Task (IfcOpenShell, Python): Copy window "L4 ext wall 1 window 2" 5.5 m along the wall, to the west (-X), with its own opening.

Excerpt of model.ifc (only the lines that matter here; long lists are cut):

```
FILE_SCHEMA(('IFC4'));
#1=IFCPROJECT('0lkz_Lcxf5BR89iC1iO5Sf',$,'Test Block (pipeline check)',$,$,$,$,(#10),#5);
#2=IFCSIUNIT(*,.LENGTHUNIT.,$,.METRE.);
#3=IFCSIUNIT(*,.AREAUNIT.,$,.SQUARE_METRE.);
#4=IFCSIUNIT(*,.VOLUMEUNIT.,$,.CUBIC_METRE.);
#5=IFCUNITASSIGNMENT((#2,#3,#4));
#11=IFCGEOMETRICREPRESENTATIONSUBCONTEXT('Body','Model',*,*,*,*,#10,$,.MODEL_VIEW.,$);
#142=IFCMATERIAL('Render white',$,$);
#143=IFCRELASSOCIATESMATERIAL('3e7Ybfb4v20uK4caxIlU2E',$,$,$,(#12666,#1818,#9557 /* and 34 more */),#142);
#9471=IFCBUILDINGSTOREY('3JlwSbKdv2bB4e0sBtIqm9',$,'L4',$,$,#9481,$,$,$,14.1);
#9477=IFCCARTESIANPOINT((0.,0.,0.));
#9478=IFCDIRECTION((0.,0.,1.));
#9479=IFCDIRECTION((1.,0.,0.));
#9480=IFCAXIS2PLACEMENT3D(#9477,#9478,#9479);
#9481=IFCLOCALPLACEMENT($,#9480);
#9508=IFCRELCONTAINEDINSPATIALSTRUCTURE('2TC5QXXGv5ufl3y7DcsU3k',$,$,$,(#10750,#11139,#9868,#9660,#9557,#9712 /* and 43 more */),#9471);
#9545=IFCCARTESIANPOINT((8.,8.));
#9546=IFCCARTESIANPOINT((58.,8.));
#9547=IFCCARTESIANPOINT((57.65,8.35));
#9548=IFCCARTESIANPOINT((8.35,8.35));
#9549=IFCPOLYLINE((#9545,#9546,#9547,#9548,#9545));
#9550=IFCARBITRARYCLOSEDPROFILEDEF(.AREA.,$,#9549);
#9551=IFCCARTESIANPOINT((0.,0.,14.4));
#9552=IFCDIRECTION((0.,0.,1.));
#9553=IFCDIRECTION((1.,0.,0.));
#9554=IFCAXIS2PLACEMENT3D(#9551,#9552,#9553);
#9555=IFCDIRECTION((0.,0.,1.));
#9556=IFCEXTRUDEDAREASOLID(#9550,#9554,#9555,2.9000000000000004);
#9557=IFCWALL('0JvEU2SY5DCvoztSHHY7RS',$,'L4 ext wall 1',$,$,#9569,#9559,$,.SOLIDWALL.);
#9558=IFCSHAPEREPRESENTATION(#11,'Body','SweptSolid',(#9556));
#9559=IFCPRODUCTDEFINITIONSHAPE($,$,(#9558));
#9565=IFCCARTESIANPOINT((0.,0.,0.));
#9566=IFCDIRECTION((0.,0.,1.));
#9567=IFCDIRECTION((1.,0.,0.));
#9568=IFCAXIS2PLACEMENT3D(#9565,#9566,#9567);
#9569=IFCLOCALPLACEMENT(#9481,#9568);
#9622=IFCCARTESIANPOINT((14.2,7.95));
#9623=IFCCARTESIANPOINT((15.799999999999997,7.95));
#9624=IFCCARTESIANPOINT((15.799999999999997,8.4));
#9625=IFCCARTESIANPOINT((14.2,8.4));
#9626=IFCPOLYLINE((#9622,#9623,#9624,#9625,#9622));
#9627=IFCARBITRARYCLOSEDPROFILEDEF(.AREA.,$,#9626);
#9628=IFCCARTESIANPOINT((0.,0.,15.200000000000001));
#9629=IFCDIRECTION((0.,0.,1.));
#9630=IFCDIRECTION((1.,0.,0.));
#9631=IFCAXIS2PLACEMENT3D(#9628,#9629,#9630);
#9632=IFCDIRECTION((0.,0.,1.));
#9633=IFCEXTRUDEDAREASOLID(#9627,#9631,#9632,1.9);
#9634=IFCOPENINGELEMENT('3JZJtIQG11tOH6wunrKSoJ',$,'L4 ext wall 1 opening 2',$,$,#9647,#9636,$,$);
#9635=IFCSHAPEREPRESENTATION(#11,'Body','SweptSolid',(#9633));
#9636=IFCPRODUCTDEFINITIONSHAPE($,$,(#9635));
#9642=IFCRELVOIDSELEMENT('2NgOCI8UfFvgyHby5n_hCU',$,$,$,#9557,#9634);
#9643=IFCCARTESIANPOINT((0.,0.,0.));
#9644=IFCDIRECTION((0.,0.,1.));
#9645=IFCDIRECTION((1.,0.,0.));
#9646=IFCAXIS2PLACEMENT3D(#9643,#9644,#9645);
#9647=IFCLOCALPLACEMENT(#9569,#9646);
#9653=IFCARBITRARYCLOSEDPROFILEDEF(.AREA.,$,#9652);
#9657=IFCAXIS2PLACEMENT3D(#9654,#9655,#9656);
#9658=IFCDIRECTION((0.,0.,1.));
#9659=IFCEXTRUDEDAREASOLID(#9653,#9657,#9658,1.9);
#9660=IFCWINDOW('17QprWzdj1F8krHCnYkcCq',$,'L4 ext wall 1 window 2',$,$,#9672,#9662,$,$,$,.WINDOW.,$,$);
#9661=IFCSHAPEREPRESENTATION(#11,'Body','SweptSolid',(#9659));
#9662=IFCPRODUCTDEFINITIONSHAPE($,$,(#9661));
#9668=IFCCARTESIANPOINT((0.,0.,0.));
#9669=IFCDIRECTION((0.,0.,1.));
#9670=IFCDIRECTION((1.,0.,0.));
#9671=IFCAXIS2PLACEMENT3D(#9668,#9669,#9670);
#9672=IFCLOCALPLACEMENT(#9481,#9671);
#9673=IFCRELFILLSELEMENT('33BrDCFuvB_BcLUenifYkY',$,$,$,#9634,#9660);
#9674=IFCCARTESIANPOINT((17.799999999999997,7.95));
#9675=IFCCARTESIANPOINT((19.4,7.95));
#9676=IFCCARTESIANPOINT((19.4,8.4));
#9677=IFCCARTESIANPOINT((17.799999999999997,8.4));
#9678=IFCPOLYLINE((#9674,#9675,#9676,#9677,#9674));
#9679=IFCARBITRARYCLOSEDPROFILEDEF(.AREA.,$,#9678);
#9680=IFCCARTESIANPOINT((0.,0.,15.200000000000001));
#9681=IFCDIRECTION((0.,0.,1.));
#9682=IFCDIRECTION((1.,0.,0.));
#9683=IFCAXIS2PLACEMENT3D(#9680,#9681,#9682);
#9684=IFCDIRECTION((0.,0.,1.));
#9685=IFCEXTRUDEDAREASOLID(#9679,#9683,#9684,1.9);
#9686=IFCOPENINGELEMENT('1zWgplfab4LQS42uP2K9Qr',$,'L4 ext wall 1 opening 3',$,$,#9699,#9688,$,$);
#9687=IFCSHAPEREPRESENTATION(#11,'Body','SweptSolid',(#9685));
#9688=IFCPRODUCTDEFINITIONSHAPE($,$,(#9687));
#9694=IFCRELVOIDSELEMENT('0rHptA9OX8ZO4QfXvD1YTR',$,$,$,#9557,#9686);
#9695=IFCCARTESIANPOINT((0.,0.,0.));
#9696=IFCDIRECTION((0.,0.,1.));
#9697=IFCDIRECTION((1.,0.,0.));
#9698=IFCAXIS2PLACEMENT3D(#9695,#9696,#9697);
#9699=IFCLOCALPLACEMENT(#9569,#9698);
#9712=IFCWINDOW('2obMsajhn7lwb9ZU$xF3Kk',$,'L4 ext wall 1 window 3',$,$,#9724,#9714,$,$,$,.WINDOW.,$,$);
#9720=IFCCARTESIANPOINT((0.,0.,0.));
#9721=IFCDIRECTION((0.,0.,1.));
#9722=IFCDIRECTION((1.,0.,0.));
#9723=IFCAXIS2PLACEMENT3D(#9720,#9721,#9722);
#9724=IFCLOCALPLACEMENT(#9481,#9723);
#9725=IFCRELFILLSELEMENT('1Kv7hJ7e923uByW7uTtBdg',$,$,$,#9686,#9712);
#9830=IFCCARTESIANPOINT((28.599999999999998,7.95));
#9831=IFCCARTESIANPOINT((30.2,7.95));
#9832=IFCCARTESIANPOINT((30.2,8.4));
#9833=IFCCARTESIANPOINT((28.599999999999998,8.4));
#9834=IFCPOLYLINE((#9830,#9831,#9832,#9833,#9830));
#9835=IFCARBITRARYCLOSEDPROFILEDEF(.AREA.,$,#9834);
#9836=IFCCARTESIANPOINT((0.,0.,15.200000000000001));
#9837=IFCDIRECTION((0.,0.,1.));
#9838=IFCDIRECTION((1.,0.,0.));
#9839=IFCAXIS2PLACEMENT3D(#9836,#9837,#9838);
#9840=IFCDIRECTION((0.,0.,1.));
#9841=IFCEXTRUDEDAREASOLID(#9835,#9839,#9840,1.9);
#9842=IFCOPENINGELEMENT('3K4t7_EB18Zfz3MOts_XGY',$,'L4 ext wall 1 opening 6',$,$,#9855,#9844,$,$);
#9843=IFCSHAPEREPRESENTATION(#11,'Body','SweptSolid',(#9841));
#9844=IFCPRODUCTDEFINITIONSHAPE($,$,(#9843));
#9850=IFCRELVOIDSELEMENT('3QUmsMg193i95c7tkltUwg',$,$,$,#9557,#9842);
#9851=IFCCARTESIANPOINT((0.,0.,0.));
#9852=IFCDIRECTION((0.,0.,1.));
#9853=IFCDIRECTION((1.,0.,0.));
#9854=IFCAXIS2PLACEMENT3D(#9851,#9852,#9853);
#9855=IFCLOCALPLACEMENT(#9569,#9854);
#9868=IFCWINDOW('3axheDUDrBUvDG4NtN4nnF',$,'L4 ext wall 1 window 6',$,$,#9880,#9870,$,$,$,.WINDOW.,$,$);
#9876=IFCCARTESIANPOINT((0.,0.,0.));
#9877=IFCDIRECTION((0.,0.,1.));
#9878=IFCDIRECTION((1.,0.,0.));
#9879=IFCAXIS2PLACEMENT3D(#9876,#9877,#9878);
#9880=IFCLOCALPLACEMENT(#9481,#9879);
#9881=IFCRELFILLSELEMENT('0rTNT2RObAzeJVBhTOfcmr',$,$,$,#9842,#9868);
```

```python
import ifcopenshell
import ifcopenshell.api.feature
import ifcopenshell.api.geometry
import ifcopenshell.api.root
import ifcopenshell.geom
import ifcopenshell.util.element
import ifcopenshell.util.placement
import ifcopenshell.util.shape
import ifcopenshell.util.unit

model = ifcopenshell.open("model.ifc")
unit_scale = ifcopenshell.util.unit.calculate_unit_scale(model)
settings = ifcopenshell.geom.settings()


def volume(element):
    """Net volume in cubic metres, openings subtracted."""
    shape = ifcopenshell.geom.create_shape(settings, element)
    return ifcopenshell.util.shape.get_volume(shape.geometry)


window = model.by_id(9660)
opening = window.FillsVoids[0].RelatingOpeningElement
wall = opening.VoidsElements[0].RelatingBuildingElement
before = volume(wall)
shift = ifcopenshell.util.placement.get_local_placement(wall.ObjectPlacement)[:3, 0] * -5.5 / unit_scale

# copy_class copies the void relationship, type, container and properties, but no geometry.
new_opening = ifcopenshell.api.root.copy_class(model, product=opening)
new_opening.Representation = ifcopenshell.util.element.copy_deep(
    model, opening.Representation, exclude=["IfcGeometricRepresentationContext", "IfcRepresentationMap"]
)
new_window = ifcopenshell.api.root.copy_class(model, product=window)
new_window.Representation = ifcopenshell.util.element.copy_deep(
    model, window.Representation, exclude=["IfcGeometricRepresentationContext", "IfcRepresentationMap"]
)
ifcopenshell.api.feature.add_filling(model, opening=new_opening, element=new_window)

for old, new in ((opening, new_opening), (window, new_window)):
    matrix = ifcopenshell.util.placement.get_local_placement(old.ObjectPlacement)
    matrix[:3, 3] += shift
    ifcopenshell.api.geometry.edit_object_placement(model, product=new, matrix=matrix, is_si=False)

after = volume(wall)

print(f"wall volume {before:.3f} -> {after:.3f} m3")

model.write("model_v2.ifc")
```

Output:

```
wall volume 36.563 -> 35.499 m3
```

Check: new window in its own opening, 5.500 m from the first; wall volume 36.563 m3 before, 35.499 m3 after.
